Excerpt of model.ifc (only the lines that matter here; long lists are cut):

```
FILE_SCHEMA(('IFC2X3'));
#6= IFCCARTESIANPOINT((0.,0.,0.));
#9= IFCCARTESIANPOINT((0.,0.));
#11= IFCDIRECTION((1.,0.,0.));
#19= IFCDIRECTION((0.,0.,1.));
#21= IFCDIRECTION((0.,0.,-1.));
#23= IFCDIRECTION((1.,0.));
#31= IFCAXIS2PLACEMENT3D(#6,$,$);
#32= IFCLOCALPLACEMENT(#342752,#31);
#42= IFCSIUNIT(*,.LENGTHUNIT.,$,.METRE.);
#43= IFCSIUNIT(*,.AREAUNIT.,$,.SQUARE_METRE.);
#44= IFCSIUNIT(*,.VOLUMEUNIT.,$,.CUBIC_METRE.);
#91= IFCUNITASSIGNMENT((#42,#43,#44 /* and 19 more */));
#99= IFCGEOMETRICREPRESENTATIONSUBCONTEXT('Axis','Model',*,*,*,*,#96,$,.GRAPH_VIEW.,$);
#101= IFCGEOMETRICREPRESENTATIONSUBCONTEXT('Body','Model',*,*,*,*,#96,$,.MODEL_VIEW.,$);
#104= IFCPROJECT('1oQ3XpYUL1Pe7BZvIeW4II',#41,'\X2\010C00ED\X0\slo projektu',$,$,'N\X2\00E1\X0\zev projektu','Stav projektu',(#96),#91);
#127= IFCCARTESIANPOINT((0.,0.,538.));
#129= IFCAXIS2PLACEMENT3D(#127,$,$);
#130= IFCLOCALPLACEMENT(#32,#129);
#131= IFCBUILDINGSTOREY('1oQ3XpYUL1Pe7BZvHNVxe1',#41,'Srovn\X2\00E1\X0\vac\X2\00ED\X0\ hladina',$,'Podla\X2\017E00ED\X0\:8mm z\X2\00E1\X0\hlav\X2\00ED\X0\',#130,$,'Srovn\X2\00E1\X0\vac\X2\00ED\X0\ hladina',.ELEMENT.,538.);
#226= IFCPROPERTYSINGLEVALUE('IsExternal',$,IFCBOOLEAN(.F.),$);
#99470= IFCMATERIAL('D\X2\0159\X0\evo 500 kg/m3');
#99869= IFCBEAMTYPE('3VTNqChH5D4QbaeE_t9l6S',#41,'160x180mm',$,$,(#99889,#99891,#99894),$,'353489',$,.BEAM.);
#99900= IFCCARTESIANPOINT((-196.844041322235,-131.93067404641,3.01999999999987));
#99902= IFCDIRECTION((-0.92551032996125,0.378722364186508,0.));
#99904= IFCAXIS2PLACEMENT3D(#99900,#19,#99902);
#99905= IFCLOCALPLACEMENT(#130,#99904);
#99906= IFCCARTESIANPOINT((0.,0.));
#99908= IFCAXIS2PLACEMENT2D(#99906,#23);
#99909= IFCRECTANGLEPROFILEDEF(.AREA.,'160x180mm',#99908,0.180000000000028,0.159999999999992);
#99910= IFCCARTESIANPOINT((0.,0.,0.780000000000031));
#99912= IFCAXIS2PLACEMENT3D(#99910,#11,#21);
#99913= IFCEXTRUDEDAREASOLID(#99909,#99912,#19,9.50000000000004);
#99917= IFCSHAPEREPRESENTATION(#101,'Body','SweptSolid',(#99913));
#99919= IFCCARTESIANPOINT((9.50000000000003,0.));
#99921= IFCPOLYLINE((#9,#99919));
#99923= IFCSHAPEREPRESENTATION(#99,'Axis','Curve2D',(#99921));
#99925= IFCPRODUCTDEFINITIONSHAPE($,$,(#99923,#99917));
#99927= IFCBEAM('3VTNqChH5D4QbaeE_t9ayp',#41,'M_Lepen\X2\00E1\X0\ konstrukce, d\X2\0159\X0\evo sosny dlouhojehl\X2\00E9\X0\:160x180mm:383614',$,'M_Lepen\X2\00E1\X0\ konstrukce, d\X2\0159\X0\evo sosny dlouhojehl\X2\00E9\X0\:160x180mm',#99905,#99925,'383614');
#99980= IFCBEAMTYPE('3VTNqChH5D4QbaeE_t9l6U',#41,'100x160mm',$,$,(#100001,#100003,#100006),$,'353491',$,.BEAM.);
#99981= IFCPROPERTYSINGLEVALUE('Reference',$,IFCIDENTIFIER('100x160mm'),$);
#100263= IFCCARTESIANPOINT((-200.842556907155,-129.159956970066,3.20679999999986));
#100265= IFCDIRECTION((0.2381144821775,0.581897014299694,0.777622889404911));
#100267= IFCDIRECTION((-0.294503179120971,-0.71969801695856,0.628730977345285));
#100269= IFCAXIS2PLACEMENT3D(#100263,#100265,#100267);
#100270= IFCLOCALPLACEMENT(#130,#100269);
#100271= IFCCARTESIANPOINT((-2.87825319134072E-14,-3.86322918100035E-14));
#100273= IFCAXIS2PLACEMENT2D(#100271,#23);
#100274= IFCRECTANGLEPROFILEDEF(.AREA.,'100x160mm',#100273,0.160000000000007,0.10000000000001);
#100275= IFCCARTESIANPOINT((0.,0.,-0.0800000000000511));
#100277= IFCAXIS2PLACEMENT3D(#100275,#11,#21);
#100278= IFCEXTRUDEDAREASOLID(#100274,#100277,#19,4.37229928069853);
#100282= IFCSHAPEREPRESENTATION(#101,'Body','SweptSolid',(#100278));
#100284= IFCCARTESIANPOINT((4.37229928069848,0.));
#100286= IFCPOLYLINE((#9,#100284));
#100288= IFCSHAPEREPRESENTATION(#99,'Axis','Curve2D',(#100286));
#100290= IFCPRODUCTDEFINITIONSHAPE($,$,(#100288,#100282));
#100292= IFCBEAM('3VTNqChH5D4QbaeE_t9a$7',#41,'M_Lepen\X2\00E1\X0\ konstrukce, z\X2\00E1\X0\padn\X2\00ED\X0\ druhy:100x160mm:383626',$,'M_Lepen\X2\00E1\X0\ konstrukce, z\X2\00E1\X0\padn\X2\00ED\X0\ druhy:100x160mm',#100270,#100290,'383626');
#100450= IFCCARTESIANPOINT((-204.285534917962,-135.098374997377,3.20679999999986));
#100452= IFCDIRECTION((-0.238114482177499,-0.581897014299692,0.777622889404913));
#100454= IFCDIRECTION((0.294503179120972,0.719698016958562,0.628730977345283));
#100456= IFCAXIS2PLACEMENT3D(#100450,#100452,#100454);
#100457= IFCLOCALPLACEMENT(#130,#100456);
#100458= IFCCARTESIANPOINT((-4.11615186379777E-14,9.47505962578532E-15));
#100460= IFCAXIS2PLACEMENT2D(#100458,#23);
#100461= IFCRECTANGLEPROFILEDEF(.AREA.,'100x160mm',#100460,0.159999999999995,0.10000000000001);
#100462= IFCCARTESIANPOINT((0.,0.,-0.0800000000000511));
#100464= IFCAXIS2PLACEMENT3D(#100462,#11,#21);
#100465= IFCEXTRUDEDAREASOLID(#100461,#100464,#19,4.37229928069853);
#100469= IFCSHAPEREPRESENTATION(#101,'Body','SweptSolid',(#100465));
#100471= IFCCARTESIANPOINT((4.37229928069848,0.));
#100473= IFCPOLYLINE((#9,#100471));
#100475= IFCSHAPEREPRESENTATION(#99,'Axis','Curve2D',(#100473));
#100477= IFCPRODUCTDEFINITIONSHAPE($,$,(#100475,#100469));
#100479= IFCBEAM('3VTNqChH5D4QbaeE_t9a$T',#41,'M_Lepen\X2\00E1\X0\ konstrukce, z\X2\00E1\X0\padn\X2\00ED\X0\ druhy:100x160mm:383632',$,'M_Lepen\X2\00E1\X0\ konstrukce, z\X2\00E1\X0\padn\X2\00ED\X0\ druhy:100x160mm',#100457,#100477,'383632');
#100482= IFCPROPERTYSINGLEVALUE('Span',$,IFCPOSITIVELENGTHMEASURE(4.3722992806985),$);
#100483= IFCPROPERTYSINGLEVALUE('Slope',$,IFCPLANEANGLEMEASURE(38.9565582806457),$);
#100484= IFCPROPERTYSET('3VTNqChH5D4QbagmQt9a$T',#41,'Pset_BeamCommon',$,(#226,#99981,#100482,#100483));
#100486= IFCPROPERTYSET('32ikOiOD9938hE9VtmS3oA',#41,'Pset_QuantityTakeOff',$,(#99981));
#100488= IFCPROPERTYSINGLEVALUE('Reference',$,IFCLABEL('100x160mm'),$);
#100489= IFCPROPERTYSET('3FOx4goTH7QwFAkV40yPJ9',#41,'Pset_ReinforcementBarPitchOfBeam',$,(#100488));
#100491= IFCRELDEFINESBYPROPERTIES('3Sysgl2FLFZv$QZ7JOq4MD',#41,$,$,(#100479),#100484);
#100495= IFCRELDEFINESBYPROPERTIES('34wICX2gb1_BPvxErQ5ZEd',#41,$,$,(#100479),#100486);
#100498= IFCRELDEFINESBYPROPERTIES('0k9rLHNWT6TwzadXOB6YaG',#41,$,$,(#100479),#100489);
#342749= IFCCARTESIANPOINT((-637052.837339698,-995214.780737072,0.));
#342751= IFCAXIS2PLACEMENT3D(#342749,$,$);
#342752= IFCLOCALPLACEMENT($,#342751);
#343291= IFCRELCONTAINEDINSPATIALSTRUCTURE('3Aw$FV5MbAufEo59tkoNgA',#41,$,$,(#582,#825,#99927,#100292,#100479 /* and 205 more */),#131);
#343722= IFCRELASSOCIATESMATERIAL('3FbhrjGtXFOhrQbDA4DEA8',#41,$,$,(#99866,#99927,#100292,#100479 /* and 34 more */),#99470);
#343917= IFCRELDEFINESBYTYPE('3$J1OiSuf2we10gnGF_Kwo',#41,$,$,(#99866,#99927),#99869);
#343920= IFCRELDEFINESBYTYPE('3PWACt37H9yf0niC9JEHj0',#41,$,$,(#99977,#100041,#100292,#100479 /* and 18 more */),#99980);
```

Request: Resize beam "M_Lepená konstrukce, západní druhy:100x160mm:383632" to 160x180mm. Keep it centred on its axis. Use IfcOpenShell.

```python
import ifcopenshell
import ifcopenshell.api.pset
import ifcopenshell.api.type
import ifcopenshell.util.element
import ifcopenshell.util.representation

model = ifcopenshell.open("model.ifc")

member = model.by_id(100479)
source = next(p for p in model.by_type("IfcRectangleProfileDef") if p.ProfileName == "160x180mm")

body = ifcopenshell.util.representation.get_representation(member, "Model", "Body")
solid = body.Items[0]
old_profile = solid.SweptArea

# Copy the section's sizes but keep this member's own profile position.
profile = ifcopenshell.util.element.copy(model, source)
profile.Position = old_profile.Position
solid.SweptArea = profile
if not model.get_total_inverses(old_profile):
    ifcopenshell.util.element.remove_deep2(model, old_profile)

new_type = model.by_guid("3VTNqChH5D4QbaeE_t9l6S")
ifcopenshell.api.type.assign_type(
    model, related_objects=[member], relating_type=new_type, should_map_representations=False
)
member.Name = member.Name.replace("100x160mm", "160x180mm")
member.ObjectType = "M_Lepená konstrukce, západní druhy:160x180mm"
pset = model.by_id(ifcopenshell.util.element.get_pset(member, "Pset_BeamCommon", should_inherit=False)["id"])
ifcopenshell.api.pset.edit_pset(model, pset=pset, properties={"Reference": "160x180mm"})
pset = model.by_id(ifcopenshell.util.element.get_pset(member, "Pset_QuantityTakeOff", should_inherit=False)["id"])
ifcopenshell.api.pset.edit_pset(model, pset=pset, properties={"Reference": "160x180mm"})
pset = model.by_id(ifcopenshell.util.element.get_pset(member, "Pset_ReinforcementBarPitchOfBeam", should_inherit=False)["id"])
ifcopenshell.api.pset.edit_pset(model, pset=pset, properties={"Reference": "160x180mm"})

print(solid.SweptArea)

model.write("model_edited.ifc")
```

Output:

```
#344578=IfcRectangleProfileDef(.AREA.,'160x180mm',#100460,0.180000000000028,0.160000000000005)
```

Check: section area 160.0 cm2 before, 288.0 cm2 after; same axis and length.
